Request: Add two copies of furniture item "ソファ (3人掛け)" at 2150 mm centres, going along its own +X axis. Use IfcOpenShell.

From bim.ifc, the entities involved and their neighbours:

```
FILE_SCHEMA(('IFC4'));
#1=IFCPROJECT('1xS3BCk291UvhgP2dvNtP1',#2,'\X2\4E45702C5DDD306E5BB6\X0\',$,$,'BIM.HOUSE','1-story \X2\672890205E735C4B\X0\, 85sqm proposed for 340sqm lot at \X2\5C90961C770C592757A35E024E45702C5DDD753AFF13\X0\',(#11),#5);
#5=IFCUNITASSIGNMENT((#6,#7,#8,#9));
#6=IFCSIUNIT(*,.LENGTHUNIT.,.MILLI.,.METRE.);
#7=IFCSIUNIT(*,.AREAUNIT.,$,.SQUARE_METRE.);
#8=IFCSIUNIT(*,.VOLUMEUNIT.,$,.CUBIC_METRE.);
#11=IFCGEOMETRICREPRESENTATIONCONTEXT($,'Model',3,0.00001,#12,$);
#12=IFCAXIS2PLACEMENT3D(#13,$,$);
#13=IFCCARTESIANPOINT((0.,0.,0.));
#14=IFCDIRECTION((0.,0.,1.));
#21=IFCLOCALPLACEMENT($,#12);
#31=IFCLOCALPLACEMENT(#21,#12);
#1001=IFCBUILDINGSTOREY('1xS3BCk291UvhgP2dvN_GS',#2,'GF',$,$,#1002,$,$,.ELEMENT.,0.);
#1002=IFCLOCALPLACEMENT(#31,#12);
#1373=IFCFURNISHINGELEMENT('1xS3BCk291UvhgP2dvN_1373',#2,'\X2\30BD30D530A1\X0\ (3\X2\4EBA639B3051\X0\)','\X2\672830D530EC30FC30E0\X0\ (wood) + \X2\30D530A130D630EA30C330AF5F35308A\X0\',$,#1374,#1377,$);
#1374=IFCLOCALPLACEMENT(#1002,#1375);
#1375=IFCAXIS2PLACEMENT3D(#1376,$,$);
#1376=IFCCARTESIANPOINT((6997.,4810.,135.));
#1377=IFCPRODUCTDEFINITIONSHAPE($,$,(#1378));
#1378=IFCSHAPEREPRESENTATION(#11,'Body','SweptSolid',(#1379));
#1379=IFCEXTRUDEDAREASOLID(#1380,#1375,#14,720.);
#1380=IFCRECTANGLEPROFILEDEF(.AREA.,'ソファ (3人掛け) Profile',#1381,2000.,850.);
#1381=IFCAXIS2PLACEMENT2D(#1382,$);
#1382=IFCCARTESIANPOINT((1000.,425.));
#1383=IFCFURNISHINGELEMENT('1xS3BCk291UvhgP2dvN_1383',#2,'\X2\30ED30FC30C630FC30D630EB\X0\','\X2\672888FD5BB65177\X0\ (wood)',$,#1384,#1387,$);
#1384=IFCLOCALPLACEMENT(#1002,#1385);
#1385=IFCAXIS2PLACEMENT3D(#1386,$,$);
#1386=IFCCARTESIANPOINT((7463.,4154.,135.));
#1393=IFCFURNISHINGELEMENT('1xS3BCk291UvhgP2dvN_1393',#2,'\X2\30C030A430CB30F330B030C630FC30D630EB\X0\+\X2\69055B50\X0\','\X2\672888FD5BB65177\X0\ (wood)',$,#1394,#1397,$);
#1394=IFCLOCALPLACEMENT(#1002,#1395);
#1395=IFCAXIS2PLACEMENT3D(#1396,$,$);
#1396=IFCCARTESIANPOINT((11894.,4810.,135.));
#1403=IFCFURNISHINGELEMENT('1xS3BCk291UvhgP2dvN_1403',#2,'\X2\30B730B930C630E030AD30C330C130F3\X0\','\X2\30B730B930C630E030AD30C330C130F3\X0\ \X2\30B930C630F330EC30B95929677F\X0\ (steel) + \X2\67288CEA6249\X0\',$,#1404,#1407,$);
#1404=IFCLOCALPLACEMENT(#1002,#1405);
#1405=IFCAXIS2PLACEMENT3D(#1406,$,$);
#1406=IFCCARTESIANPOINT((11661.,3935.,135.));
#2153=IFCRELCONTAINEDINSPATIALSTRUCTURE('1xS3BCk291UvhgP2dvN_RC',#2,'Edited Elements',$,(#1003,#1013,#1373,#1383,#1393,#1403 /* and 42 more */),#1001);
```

```python
import ifcopenshell
import ifcopenshell.api.geometry
import ifcopenshell.api.root
import ifcopenshell.util.element
import ifcopenshell.util.placement
import ifcopenshell.util.unit

model = ifcopenshell.open("bim.ifc")
unit_scale = ifcopenshell.util.unit.calculate_unit_scale(model)


def reuse_history(source, copy):
    """copy_class also copies each property set's owner history, people and application; keep the originals."""
    for rel in copy.IsDefinedBy:
        if rel.is_a("IfcRelDefinesByProperties") and (history := rel.RelatingPropertyDefinition.OwnerHistory):
            rel.RelatingPropertyDefinition.OwnerHistory = source.OwnerHistory
            ifcopenshell.util.element.remove_deep2(model, history)


source = model.by_guid("1xS3BCk291UvhgP2dvN_1373")
base = ifcopenshell.util.placement.get_local_placement(source.ObjectPlacement)
step = base[:3, 0] * 2.15 / unit_scale

for i in range(1, 3):
    copy = ifcopenshell.api.root.copy_class(model, product=source)
    copy.Representation = ifcopenshell.util.element.copy_deep(
        model, source.Representation, exclude=["IfcGeometricRepresentationContext", "IfcRepresentationMap"]
    )
    reuse_history(source, copy)
    matrix = base.copy()
    matrix[:3, 3] += i * step
    print("added at", matrix[:3, 3].round(3) + 0.0)
    ifcopenshell.api.geometry.edit_object_placement(model, product=copy, matrix=matrix, is_si=False)

model.write("bim_updated.ifc")
```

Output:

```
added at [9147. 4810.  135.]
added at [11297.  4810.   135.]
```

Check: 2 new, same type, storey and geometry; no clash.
